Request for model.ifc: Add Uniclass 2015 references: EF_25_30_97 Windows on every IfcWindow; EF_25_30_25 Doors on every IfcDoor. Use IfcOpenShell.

First a look at what the model holds.

```python
import ifcopenshell

model = ifcopenshell.open("model.ifc")
print(model.schema)
print("classifications:", [c.Name for c in model.by_type("IfcClassification")])
for ifc_class in ("IfcDoor", "IfcRoof", "IfcStair", "IfcWall", "IfcWindow"):
    print(ifc_class, len(model.by_type(ifc_class)))
```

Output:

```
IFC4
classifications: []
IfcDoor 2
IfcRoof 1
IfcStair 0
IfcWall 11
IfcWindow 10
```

```python
import ifcopenshell
import ifcopenshell.api.classification

model = ifcopenshell.open("model.ifc")

system = ifcopenshell.api.classification.add_classification(model, classification="Uniclass 2015")

codes = {
    "IfcWindow": ("EF_25_30_97", "Windows"),
    "IfcDoor": ("EF_25_30_25", "Doors"),
}
for ifc_class, (code, name) in codes.items():
    products = model.by_type(ifc_class)
    ifcopenshell.api.classification.add_reference(
        model, products=products, classification=system, identification=code, name=name
    )
    print(code, len(products))

model.write("model_edited.ifc")
```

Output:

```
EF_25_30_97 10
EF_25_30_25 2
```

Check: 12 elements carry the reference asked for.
